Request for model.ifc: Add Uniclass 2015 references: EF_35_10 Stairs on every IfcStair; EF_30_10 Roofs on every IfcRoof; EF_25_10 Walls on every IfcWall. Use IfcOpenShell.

First a look at what the model holds.

```python
import ifcopenshell

model = ifcopenshell.open("model.ifc")
print(model.schema)
print("classifications:", [c.Name for c in model.by_type("IfcClassification")])
for ifc_class in ("IfcDoor", "IfcRoof", "IfcStair", "IfcWall", "IfcWindow"):
    print(ifc_class, len(model.by_type(ifc_class)))
```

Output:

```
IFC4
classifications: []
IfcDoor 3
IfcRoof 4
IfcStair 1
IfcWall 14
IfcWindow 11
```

```python
import ifcopenshell
import ifcopenshell.api.classification

model = ifcopenshell.open("model.ifc")

system = ifcopenshell.api.classification.add_classification(model, classification="Uniclass 2015")

codes = {
    "IfcStair": ("EF_35_10", "Stairs"),
    "IfcRoof": ("EF_30_10", "Roofs"),
    "IfcWall": ("EF_25_10", "Walls"),
}
for ifc_class, (code, name) in codes.items():
    products = model.by_type(ifc_class)
    ifcopenshell.api.classification.add_reference(
        model, products=products, classification=system, identification=code, name=name
    )
    print(code, len(products))

model.write("model_v2.ifc")
```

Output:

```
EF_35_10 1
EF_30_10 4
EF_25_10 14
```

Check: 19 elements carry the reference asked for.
